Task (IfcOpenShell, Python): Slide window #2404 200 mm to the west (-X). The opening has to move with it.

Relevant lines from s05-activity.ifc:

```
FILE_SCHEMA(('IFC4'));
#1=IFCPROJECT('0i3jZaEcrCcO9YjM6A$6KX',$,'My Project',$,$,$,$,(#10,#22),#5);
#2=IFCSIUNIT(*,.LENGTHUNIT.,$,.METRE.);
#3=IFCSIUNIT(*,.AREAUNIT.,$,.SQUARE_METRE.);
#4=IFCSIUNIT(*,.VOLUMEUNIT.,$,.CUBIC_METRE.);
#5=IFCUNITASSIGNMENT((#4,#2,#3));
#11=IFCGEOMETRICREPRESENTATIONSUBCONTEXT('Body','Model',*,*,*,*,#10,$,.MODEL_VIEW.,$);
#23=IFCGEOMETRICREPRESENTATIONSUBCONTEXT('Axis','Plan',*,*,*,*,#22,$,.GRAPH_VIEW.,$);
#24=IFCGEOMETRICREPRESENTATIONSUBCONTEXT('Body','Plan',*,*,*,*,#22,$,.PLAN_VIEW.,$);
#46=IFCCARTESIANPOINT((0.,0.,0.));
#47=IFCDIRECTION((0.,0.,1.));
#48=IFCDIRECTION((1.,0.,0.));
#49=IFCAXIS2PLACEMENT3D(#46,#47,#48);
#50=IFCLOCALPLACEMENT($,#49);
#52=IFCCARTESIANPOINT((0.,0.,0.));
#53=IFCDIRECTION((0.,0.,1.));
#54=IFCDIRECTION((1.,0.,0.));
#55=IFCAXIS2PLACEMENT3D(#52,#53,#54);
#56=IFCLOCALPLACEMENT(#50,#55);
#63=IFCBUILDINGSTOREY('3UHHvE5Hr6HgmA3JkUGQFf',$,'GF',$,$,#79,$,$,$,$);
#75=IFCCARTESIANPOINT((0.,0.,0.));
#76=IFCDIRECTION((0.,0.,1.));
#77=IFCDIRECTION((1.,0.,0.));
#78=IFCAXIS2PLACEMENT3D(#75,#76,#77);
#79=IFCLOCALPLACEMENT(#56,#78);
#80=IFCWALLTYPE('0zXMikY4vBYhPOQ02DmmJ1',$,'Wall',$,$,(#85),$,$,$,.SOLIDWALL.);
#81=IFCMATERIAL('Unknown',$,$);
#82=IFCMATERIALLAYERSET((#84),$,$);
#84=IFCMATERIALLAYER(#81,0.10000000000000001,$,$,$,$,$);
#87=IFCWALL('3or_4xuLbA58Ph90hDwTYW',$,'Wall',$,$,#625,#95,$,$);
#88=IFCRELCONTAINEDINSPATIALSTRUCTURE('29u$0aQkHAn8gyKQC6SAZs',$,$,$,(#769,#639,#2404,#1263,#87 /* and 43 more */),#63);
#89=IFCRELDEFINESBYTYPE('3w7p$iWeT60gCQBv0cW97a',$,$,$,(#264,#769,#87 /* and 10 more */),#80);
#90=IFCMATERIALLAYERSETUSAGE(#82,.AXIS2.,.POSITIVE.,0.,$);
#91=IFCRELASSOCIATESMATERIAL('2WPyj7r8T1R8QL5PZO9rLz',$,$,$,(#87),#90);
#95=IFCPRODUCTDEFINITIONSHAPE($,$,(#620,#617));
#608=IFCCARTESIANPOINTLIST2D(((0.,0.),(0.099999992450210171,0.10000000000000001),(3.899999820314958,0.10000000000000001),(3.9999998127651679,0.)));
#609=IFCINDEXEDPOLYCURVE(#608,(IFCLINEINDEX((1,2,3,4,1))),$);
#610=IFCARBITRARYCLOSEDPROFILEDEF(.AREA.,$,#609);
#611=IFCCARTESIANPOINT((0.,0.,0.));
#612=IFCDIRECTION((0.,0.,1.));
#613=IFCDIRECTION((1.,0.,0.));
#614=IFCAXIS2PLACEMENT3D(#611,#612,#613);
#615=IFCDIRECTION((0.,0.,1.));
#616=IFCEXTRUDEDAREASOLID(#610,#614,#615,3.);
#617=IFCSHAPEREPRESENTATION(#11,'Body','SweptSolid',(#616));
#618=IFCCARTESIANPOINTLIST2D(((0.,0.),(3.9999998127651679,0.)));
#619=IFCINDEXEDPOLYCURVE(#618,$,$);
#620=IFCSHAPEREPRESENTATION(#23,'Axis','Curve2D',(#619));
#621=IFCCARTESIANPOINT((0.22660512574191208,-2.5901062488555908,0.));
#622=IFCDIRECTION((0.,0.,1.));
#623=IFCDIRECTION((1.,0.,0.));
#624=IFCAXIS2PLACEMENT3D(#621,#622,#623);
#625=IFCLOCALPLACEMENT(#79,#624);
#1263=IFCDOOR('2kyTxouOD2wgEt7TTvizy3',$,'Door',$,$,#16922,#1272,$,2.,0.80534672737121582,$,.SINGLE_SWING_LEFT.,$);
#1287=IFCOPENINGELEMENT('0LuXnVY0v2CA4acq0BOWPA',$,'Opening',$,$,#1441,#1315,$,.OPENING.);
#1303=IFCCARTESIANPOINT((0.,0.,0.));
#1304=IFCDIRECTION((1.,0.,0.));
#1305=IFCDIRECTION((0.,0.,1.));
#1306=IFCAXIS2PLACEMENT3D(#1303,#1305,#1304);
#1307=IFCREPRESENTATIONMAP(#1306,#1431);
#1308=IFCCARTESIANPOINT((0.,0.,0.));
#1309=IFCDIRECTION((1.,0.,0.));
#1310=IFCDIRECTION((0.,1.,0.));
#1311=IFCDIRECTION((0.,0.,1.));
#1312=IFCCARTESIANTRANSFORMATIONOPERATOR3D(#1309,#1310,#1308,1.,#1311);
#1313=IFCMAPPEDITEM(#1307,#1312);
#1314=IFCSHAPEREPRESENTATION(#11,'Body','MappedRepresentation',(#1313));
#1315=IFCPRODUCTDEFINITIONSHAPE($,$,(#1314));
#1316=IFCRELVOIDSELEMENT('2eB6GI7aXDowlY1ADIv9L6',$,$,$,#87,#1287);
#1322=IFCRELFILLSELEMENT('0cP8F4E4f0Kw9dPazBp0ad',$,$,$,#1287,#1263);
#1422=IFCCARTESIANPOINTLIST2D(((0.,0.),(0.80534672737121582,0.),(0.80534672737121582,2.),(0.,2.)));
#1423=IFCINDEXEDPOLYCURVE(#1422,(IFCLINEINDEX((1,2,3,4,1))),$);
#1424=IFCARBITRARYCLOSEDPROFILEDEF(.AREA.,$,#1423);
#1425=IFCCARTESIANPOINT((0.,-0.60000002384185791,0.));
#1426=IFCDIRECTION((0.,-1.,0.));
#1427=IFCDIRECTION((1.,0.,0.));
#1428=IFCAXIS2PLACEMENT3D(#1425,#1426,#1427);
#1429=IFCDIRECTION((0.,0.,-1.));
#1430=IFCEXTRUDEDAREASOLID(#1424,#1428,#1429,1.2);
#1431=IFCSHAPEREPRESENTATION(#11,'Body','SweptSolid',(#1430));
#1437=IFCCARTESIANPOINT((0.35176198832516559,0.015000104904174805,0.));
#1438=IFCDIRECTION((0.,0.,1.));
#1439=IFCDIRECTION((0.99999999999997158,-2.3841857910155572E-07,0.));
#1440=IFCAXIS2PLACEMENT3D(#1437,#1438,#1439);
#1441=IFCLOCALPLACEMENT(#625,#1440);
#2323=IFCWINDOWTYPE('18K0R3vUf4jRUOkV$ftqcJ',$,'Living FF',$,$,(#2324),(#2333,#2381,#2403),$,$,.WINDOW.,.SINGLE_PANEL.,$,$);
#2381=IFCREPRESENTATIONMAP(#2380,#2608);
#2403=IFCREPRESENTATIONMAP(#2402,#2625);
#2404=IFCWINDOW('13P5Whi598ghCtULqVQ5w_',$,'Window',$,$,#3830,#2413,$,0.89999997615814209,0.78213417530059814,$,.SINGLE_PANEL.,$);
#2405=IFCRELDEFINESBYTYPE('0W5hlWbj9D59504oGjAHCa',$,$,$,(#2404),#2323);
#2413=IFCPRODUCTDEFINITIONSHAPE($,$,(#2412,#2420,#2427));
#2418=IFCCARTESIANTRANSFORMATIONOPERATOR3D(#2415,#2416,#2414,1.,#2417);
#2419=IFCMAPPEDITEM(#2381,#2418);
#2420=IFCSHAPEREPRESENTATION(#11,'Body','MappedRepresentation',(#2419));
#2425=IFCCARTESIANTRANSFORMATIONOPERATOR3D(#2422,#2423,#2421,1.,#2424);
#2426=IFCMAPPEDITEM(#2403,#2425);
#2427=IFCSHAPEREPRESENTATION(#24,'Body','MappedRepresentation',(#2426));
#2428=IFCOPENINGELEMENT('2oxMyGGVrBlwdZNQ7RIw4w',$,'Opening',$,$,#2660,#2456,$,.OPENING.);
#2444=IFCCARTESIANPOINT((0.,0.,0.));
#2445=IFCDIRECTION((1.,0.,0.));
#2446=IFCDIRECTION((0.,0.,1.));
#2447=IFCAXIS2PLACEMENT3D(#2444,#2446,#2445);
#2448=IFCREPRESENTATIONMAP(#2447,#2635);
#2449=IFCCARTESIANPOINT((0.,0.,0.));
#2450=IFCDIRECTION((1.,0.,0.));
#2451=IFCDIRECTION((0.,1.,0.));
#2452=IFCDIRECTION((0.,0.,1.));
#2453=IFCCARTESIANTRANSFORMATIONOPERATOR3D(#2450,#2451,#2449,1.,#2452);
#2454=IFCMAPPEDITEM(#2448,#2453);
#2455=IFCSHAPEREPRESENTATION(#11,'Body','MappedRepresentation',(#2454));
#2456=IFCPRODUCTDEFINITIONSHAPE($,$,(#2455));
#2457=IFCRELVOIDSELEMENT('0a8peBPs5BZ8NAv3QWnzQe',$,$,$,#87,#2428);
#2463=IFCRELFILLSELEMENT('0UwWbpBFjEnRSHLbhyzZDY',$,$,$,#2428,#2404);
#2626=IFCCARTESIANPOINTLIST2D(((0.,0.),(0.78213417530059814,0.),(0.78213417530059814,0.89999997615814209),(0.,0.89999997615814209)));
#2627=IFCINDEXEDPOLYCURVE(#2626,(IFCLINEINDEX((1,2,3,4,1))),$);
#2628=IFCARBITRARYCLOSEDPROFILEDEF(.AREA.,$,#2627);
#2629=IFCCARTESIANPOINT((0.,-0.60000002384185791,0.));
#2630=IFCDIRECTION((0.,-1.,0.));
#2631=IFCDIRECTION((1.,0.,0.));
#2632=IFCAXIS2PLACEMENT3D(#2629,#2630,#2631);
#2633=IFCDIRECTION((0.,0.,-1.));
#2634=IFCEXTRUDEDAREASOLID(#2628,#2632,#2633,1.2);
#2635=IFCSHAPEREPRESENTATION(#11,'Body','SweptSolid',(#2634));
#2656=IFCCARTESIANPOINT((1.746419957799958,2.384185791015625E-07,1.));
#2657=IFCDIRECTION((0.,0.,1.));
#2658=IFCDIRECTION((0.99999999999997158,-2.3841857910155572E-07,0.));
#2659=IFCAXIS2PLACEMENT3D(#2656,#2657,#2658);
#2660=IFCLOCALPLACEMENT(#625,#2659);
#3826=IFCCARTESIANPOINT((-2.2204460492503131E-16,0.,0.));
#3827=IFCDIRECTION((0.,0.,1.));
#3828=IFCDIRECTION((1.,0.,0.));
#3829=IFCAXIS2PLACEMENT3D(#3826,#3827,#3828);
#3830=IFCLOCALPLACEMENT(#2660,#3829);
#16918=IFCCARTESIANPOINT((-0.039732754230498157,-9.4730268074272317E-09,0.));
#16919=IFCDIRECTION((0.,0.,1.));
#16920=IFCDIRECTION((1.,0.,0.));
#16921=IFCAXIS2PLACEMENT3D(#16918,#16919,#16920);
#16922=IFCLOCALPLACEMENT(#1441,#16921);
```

```python
import ifcopenshell
import ifcopenshell.api.geometry
import ifcopenshell.util.placement
import ifcopenshell.util.unit

model = ifcopenshell.open("s05-activity.ifc")
unit_scale = ifcopenshell.util.unit.calculate_unit_scale(model)

window = model.by_id(2404)
opening = window.FillsVoids[0].RelatingOpeningElement
wall = opening.VoidsElements[0].RelatingBuildingElement

wall_matrix = ifcopenshell.util.placement.get_local_placement(wall.ObjectPlacement)
shift = wall_matrix[:3, 0] * -0.2 / unit_scale
before = ifcopenshell.util.placement.get_local_placement(window.ObjectPlacement)[:3, 3].copy()

# The window is placed relative to its opening, so it follows when the opening moves.
matrix = ifcopenshell.util.placement.get_local_placement(opening.ObjectPlacement)
matrix[:3, 3] += shift
ifcopenshell.api.geometry.edit_object_placement(
    model, product=opening, matrix=matrix, is_si=False, should_transform_children=True
)

after = ifcopenshell.util.placement.get_local_placement(window.ObjectPlacement)[:3, 3]
print("window moved by", (after - before).round(3) + 0.0)

model.write("s05-activity_v2.ifc")
```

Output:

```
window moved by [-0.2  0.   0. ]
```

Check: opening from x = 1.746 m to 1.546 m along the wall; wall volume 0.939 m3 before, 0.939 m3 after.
